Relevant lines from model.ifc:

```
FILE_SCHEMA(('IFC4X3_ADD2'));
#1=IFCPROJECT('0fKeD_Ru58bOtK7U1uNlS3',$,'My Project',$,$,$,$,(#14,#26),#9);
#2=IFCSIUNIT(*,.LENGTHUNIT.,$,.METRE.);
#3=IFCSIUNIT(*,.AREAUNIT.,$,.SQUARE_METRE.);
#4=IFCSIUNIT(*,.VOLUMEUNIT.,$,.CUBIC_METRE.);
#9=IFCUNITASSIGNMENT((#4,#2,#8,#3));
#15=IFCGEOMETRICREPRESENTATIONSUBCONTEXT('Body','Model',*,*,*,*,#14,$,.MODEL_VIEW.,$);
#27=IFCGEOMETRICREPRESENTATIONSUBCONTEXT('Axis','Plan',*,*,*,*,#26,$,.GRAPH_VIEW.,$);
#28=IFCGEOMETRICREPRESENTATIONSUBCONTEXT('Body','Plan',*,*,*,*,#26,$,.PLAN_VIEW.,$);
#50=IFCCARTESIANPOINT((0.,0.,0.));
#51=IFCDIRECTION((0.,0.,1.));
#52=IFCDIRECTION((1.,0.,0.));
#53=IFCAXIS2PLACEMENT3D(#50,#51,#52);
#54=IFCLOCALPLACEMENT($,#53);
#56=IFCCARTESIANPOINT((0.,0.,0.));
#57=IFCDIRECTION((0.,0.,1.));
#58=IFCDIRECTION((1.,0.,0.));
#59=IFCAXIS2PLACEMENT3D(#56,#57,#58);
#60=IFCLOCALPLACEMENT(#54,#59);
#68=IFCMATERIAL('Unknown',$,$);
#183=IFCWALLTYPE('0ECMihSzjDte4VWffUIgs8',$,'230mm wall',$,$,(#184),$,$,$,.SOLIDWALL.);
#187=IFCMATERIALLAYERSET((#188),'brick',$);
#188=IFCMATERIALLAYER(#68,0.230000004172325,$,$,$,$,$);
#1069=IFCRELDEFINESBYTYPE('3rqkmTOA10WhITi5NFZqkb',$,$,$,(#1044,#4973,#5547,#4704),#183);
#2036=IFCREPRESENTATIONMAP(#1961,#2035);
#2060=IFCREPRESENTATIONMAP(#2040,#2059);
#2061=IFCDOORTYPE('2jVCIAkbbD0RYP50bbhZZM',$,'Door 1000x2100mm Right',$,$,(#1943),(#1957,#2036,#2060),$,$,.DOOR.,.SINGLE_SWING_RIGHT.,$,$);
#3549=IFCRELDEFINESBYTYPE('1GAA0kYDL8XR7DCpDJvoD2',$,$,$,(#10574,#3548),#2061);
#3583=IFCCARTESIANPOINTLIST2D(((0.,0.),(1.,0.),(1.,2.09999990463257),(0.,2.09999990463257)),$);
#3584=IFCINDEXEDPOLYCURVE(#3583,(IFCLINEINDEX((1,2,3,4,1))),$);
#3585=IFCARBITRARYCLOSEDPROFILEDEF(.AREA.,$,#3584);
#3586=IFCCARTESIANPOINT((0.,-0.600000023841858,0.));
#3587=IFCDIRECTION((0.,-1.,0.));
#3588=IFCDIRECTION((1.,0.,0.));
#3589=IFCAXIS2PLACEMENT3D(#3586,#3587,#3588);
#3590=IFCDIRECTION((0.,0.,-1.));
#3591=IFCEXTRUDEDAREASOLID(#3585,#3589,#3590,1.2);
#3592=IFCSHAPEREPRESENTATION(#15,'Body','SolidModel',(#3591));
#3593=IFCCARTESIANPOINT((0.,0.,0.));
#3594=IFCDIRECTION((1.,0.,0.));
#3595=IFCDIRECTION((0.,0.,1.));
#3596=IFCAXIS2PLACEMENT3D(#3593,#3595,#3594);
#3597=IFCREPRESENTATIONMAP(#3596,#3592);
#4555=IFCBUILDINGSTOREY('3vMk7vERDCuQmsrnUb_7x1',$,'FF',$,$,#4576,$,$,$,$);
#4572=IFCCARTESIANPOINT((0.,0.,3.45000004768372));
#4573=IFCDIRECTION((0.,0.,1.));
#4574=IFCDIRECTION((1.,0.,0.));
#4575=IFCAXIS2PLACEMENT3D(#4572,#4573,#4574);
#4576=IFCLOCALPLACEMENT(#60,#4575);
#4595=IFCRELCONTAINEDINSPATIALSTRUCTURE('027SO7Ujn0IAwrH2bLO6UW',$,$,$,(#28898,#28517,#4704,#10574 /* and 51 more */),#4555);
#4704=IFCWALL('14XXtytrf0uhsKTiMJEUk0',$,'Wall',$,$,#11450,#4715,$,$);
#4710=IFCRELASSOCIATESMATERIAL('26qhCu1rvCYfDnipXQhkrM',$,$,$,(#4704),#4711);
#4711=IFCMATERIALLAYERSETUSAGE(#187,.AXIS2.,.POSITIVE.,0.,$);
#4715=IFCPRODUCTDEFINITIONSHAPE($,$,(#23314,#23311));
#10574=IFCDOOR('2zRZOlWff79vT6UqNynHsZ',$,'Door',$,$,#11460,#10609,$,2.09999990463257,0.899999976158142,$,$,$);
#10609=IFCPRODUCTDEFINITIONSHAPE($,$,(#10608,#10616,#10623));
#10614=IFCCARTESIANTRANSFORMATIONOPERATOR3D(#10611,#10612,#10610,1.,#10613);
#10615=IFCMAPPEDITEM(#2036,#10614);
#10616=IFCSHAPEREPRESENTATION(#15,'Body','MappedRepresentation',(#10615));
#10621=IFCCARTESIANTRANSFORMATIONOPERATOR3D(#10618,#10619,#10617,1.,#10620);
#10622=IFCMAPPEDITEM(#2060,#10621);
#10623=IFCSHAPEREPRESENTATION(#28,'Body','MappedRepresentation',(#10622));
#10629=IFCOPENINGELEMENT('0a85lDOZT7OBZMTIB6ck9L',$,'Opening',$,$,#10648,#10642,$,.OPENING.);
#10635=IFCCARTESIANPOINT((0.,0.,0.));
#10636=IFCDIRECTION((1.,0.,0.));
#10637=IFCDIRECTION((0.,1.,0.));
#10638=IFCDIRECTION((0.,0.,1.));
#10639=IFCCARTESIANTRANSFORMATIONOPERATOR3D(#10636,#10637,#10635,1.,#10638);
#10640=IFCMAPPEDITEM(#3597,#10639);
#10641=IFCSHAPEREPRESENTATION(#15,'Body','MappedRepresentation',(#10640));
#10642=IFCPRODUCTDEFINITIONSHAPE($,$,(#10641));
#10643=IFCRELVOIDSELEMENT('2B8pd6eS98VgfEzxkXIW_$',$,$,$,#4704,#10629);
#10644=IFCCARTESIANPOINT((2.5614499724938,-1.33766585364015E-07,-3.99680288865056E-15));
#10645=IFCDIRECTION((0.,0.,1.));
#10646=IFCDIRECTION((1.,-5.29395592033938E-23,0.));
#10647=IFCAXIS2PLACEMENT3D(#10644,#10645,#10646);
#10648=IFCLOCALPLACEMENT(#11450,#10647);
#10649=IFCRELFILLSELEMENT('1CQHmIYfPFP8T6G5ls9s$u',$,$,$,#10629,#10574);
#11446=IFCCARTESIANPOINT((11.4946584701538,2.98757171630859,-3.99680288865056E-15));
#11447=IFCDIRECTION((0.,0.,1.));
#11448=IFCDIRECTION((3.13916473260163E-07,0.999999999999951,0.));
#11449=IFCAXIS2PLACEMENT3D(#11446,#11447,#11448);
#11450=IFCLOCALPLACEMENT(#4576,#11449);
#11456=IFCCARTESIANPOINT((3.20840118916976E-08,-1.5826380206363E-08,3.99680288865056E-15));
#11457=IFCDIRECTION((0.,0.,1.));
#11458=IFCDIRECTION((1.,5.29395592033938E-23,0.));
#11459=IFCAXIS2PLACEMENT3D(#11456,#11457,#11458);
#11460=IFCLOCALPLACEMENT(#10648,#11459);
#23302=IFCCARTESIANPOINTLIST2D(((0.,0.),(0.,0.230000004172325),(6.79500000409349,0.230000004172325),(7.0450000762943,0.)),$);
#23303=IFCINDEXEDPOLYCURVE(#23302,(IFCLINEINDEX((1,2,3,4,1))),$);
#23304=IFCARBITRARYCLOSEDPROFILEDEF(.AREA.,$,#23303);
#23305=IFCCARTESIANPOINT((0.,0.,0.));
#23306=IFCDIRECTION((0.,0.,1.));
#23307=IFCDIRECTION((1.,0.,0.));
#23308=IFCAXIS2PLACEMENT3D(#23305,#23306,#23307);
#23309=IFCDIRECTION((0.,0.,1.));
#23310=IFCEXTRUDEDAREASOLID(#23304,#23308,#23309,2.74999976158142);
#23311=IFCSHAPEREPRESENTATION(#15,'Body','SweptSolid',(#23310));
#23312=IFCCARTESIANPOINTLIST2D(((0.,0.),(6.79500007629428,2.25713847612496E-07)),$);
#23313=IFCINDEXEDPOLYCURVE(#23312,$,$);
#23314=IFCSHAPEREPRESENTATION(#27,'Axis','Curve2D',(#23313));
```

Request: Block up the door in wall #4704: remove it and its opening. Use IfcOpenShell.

```python
import ifcopenshell
import ifcopenshell.api.feature
import ifcopenshell.api.root
import ifcopenshell.geom
import ifcopenshell.util.shape

model = ifcopenshell.open("model.ifc")
settings = ifcopenshell.geom.settings()


def volume(element):
    """Net volume in cubic metres, openings subtracted."""
    shape = ifcopenshell.geom.create_shape(settings, element)
    return ifcopenshell.util.shape.get_volume(shape.geometry)


door = model.by_guid("2zRZOlWff79vT6UqNynHsZ")
opening = door.FillsVoids[0].RelatingOpeningElement
wall = opening.VoidsElements[0].RelatingBuildingElement
before = volume(wall)

ifcopenshell.api.root.remove_product(model, product=door)
ifcopenshell.api.feature.remove_feature(model, feature=opening)

after = volume(wall)

print(f"wall volume {before:.3f} -> {after:.3f} m3")

model.write("model_rev.ifc")
```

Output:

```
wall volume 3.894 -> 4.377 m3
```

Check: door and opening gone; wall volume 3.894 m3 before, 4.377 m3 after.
